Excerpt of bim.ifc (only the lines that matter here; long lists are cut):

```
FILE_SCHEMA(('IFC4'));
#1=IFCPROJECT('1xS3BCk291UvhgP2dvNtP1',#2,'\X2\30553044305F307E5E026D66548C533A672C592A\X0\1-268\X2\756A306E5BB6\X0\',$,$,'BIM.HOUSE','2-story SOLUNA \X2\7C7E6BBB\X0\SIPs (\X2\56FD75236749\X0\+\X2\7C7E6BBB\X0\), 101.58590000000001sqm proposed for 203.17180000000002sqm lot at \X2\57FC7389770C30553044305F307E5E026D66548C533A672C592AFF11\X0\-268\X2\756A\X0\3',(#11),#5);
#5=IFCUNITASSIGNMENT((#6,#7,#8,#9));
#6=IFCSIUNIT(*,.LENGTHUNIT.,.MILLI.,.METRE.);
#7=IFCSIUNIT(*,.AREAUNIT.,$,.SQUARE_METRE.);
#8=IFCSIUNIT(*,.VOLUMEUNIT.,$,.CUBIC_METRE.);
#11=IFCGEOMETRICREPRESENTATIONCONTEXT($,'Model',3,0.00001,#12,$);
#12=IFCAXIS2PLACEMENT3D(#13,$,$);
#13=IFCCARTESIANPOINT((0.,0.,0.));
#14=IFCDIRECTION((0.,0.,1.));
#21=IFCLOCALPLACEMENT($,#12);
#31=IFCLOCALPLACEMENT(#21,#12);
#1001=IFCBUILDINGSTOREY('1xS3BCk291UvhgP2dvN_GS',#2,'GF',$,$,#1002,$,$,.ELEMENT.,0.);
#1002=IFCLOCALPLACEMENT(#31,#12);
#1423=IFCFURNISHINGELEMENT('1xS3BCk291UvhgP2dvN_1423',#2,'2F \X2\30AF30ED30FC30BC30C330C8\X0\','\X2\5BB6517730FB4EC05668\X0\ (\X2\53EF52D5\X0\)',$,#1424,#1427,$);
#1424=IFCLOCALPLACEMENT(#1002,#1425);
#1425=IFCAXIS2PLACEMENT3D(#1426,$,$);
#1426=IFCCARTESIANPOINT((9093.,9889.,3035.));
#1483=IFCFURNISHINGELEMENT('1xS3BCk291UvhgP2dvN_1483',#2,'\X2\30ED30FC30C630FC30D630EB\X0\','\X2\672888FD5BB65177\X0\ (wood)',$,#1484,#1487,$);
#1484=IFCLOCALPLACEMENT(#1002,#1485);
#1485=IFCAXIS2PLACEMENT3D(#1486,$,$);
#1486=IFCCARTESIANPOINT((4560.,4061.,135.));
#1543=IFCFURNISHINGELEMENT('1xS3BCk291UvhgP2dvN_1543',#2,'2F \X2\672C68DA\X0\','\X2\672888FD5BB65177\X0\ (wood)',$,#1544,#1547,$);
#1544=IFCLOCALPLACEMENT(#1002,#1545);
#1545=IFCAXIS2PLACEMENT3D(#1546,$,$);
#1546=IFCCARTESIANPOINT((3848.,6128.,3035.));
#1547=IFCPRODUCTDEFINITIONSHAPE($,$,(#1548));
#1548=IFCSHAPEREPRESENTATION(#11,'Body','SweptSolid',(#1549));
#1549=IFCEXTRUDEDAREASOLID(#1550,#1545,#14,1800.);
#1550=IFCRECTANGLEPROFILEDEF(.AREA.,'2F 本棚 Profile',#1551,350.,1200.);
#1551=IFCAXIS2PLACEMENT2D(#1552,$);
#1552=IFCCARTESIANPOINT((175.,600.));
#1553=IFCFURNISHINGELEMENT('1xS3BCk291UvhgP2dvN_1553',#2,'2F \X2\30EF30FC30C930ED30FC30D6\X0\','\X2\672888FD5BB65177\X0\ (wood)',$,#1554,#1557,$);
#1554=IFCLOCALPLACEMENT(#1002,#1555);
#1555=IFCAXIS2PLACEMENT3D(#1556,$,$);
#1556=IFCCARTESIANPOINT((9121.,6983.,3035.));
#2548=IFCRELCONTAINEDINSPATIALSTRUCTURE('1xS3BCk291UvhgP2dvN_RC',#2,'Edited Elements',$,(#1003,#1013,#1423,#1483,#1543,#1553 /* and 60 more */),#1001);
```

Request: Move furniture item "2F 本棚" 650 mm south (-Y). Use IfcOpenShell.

```python
import ifcopenshell
import ifcopenshell.api.geometry
import ifcopenshell.util.placement
import ifcopenshell.util.unit

model = ifcopenshell.open("bim.ifc")
unit_scale = ifcopenshell.util.unit.calculate_unit_scale(model)

item = model.by_guid("1xS3BCk291UvhgP2dvN_1543")
matrix = ifcopenshell.util.placement.get_local_placement(item.ObjectPlacement)
matrix[1, 3] -= 0.65 / unit_scale
ifcopenshell.api.geometry.edit_object_placement(model, product=item, matrix=matrix, is_si=False)

print(ifcopenshell.util.placement.get_local_placement(item.ObjectPlacement).round(3) + 0.0)

model.write("bim_edited.ifc")
```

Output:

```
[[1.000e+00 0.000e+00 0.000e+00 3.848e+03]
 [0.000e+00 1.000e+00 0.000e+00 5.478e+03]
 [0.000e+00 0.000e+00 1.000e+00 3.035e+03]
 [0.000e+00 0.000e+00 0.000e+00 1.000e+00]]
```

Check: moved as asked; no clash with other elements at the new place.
